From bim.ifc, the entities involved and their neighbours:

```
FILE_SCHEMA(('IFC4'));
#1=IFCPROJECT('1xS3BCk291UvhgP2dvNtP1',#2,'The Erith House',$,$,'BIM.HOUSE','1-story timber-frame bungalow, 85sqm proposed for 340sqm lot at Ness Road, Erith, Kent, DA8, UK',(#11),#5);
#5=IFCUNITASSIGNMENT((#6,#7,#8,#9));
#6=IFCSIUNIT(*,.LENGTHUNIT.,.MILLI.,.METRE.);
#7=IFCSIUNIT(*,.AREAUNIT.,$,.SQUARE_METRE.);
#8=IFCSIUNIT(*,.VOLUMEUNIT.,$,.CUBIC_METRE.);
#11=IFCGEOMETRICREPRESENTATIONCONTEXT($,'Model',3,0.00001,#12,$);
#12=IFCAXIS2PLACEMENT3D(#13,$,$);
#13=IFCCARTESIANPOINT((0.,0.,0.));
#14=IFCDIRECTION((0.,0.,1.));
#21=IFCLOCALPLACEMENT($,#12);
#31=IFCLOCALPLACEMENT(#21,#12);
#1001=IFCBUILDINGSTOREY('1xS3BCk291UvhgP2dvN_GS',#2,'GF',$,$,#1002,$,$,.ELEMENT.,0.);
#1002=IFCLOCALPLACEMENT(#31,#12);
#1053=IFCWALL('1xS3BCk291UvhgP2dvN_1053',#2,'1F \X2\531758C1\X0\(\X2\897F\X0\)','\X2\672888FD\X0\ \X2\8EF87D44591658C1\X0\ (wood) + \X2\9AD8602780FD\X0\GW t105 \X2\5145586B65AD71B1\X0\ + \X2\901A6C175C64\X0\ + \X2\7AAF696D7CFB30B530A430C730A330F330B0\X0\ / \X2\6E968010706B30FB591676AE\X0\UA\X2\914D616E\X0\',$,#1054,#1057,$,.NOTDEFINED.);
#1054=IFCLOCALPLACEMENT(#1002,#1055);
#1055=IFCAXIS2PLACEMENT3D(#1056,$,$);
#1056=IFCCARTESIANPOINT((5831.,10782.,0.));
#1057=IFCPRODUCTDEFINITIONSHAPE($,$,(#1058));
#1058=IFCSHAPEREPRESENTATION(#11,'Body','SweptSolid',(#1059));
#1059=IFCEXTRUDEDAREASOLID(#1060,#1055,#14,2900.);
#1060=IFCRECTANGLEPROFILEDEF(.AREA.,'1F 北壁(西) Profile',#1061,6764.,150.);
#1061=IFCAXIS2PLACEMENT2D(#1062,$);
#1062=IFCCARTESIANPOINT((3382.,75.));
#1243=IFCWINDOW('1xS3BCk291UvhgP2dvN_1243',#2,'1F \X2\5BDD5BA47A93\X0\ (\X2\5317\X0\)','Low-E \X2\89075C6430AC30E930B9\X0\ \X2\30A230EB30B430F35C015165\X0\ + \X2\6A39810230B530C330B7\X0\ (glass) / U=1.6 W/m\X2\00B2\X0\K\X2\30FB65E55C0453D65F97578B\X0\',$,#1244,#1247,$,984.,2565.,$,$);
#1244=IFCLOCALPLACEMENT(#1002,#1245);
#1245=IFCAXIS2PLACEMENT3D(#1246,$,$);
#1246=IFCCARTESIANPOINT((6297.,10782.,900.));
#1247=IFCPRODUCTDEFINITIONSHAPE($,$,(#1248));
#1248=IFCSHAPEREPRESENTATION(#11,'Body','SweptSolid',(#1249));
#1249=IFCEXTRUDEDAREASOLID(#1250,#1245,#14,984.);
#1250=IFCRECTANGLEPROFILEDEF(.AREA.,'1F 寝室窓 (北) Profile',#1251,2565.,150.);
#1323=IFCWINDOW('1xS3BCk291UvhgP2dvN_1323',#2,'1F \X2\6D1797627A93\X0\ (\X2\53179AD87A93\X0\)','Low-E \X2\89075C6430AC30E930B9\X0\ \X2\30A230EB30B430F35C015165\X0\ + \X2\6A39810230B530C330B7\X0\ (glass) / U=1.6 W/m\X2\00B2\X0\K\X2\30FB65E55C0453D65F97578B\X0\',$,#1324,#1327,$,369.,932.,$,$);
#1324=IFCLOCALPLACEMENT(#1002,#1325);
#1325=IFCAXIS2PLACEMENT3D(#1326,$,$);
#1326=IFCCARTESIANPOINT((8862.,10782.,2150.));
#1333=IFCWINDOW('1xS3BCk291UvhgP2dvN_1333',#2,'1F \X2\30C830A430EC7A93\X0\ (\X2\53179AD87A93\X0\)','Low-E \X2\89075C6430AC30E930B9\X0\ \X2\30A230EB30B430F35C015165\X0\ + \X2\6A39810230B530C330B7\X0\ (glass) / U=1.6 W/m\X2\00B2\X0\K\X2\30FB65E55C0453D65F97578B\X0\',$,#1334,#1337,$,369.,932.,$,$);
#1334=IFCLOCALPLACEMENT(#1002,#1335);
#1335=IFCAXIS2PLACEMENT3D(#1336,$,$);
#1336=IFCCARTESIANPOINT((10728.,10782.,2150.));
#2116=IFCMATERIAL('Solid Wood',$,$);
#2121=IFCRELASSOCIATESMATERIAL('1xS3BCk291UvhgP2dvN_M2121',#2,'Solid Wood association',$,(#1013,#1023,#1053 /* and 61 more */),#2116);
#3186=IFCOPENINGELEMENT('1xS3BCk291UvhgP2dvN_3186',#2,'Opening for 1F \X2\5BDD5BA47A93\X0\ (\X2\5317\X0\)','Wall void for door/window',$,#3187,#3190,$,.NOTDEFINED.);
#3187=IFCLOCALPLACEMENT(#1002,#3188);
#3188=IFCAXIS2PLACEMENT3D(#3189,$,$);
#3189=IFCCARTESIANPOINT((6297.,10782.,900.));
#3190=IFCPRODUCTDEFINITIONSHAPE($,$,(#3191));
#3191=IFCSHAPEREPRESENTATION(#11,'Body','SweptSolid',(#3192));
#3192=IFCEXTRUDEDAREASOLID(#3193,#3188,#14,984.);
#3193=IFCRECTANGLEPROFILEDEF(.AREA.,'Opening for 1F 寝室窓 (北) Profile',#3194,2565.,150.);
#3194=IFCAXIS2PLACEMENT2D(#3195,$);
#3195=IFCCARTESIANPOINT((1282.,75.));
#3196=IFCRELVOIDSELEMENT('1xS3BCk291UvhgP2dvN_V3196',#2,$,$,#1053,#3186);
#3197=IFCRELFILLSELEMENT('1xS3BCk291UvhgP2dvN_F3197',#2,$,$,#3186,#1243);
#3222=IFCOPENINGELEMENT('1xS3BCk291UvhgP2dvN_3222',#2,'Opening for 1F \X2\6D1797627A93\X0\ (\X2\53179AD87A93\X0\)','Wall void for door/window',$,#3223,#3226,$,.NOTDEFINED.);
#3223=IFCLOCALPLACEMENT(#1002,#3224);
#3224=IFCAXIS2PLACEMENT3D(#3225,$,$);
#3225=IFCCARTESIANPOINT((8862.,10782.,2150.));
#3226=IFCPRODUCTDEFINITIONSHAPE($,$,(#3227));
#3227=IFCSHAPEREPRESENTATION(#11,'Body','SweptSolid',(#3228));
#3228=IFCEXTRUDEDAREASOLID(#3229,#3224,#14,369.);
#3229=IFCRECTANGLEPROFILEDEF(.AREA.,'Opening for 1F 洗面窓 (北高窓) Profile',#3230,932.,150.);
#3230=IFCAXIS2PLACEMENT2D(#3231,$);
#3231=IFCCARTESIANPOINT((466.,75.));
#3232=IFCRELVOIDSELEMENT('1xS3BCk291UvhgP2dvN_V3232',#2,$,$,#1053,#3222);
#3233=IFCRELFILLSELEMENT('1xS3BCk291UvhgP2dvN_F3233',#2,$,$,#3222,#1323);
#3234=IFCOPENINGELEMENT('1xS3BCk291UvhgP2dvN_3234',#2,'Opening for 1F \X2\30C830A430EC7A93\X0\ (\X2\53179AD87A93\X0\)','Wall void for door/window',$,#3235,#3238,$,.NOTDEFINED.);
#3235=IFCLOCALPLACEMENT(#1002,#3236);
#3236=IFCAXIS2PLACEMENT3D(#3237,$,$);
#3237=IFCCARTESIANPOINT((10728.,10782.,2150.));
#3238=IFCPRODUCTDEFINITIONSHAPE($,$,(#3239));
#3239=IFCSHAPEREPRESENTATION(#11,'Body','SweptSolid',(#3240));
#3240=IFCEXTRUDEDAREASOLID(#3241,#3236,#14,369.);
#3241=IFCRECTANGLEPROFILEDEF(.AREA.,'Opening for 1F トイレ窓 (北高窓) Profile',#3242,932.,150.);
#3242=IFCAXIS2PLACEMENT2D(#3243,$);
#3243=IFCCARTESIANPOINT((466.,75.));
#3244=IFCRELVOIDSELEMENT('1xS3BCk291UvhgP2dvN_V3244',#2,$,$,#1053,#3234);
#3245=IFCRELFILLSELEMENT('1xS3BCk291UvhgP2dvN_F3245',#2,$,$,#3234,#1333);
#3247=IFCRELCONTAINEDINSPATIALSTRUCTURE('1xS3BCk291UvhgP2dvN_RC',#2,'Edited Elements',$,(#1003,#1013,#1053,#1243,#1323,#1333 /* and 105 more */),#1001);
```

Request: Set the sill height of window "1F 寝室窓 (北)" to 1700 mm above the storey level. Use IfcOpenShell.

```python
import numpy as np
import ifcopenshell
import ifcopenshell.api.geometry
import ifcopenshell.geom
import ifcopenshell.util.element
import ifcopenshell.util.placement
import ifcopenshell.util.shape
import ifcopenshell.util.unit

model = ifcopenshell.open("bim.ifc")
unit_scale = ifcopenshell.util.unit.calculate_unit_scale(model)

window = model.by_guid("1xS3BCk291UvhgP2dvN_1243")
opening = window.FillsVoids[0].RelatingOpeningElement
storey = ifcopenshell.util.element.get_container(window, ifc_class="IfcBuildingStorey")
level = ifcopenshell.util.placement.get_local_placement(storey.ObjectPlacement)[2, 3]

# The opening's origin need not be at the sill, so measure its lowest point.
shape = ifcopenshell.geom.create_shape(ifcopenshell.geom.settings(), opening)
bottom = ifcopenshell.util.shape.get_shape_bottom_elevation(shape, shape.geometry) / unit_scale
dz = level + 1.7 / unit_scale - bottom

shift = np.array([0.0, 0.0, dz])
# The window is not placed relative to its opening, so move both.
for product in (opening, window):
    matrix = ifcopenshell.util.placement.get_local_placement(product.ObjectPlacement)
    matrix[:3, 3] += shift
    ifcopenshell.api.geometry.edit_object_placement(model, product=product, matrix=matrix, is_si=False)

print(f"moved by {dz * unit_scale:+.3f} m")

model.write("bim_updated.ifc")
```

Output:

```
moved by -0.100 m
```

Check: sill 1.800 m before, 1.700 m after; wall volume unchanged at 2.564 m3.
